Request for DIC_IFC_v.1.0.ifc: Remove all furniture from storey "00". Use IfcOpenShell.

First a look at what the model holds.

```python
import ifcopenshell
import ifcopenshell.util.element

model = ifcopenshell.open("DIC_IFC_v.1.0.ifc")
print(model.schema)
storey = next(s for s in model.by_type("IfcBuildingStorey") if s.Name == "00")
furniture = [e for e in ifcopenshell.util.element.get_decomposition(storey) if e.is_a("IfcFurnishingElement")]
seen = {}
for e in furniture:
    element_type = ifcopenshell.util.element.get_type(e)
    name = element_type.Name if element_type not in (None, e) else None
    seen[name] = seen.get(name, 0) + 1
for name, count in sorted(seen.items(), key=str):
    print(count, "x", name)
```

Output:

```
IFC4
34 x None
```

```python
import ifcopenshell
import ifcopenshell.api.root
import ifcopenshell.util.element

model = ifcopenshell.open("DIC_IFC_v.1.0.ifc")

storey = next(s for s in model.by_type("IfcBuildingStorey") if s.Name == "00")
furniture = [e for e in ifcopenshell.util.element.get_decomposition(storey) if e.is_a("IfcFurnishingElement")]

for e in furniture:
    ifcopenshell.api.root.remove_product(model, product=e)
print(len(furniture), "removed")

model.write("DIC_IFC_v.1.0_rev.ifc")
```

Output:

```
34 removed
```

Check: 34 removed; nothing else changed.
